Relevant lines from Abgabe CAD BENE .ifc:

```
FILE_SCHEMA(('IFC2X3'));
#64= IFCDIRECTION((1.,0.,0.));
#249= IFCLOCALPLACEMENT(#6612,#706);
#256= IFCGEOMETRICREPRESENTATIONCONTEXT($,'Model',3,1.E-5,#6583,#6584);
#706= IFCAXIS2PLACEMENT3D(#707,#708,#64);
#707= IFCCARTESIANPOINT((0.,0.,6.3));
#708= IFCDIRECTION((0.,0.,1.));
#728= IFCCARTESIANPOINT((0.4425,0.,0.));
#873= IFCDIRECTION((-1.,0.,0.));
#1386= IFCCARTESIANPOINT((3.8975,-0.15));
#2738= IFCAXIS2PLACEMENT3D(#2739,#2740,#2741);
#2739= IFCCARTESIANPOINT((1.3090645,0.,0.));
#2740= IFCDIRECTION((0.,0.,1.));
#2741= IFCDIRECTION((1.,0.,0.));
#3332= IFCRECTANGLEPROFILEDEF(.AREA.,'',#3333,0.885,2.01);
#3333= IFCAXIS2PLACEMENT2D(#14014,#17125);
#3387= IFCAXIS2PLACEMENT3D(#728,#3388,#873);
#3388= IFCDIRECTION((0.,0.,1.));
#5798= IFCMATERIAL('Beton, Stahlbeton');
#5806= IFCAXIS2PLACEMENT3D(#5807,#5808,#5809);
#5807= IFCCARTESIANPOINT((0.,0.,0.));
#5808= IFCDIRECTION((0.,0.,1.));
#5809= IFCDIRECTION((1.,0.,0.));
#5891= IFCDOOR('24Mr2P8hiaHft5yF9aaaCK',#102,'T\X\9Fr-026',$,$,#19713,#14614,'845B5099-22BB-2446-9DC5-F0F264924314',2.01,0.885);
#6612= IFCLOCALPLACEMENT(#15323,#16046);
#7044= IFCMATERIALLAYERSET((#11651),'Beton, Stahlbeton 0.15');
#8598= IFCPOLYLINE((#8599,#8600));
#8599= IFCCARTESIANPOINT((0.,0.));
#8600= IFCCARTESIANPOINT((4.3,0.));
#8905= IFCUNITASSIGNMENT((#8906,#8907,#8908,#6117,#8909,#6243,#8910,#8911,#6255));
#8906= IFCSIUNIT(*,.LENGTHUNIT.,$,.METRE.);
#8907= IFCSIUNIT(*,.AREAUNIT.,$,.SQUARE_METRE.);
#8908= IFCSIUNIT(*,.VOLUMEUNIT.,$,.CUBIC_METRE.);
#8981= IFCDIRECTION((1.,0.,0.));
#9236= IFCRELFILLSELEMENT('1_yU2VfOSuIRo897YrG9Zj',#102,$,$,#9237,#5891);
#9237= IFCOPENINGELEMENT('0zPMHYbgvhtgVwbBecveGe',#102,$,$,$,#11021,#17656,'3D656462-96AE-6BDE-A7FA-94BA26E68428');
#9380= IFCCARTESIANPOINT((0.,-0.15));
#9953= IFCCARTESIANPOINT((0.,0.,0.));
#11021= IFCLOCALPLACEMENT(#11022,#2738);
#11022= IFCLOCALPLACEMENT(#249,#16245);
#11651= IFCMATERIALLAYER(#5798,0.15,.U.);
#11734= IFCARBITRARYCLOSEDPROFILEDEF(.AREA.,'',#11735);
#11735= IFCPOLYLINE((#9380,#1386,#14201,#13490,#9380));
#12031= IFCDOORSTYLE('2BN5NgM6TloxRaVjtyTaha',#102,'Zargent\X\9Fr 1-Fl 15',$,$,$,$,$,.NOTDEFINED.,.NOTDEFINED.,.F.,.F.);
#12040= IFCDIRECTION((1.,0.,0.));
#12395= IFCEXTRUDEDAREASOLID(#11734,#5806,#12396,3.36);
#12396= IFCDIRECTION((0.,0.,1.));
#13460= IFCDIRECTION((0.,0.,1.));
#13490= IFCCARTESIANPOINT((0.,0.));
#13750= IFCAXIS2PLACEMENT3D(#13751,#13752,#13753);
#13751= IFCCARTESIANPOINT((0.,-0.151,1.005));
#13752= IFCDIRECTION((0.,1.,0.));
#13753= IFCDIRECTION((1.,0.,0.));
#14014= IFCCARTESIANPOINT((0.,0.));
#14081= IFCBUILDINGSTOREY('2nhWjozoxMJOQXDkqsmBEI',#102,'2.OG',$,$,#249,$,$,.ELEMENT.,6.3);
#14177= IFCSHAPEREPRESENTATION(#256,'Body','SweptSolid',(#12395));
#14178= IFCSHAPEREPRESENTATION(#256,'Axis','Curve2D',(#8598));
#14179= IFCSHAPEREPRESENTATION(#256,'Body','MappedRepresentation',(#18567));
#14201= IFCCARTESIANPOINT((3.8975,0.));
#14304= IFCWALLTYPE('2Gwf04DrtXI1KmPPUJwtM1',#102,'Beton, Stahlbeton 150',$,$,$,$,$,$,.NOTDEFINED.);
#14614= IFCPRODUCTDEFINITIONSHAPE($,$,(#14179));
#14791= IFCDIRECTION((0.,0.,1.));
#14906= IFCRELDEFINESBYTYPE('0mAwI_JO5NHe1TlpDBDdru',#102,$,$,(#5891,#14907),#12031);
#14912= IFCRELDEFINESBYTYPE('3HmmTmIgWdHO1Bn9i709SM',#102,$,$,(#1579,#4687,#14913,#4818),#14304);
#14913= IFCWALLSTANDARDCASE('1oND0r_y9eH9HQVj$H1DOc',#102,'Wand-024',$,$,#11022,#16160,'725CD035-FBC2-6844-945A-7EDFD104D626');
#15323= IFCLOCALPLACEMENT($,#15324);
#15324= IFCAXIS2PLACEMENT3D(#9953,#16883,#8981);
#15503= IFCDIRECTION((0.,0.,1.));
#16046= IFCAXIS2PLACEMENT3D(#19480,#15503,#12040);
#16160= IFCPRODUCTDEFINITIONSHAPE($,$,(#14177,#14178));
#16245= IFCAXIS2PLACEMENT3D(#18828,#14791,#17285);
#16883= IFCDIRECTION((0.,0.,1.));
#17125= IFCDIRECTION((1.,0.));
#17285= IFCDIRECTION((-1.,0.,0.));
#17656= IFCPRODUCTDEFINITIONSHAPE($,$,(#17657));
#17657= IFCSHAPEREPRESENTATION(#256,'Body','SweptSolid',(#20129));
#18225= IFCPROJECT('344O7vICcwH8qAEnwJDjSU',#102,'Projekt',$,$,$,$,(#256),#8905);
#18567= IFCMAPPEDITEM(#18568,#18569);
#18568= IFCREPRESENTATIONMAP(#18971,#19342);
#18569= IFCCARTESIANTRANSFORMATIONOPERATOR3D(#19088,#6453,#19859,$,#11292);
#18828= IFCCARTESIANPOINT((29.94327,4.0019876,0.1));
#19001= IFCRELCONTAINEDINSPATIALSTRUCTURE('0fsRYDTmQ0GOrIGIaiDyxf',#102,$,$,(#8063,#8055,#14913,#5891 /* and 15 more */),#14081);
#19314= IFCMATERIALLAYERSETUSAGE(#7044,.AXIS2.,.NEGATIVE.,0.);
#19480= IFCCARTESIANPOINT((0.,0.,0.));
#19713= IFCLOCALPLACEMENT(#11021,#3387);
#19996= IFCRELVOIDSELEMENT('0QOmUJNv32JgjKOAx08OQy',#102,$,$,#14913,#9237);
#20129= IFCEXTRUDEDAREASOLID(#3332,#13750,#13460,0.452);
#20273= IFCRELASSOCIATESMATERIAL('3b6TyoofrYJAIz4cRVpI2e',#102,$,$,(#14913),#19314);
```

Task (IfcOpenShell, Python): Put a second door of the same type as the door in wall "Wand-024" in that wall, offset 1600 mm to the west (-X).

```python
import ifcopenshell
import ifcopenshell.api.feature
import ifcopenshell.api.geometry
import ifcopenshell.api.root
import ifcopenshell.geom
import ifcopenshell.util.element
import ifcopenshell.util.placement
import ifcopenshell.util.shape

model = ifcopenshell.open("Abgabe CAD BENE .ifc")
settings = ifcopenshell.geom.settings()


def volume(element):
    """Net volume in cubic metres, openings subtracted."""
    shape = ifcopenshell.geom.create_shape(settings, element)
    return ifcopenshell.util.shape.get_volume(shape.geometry)


def reuse_history(source, copy):
    """copy_class also copies each property set's owner history, people and application; keep the originals."""
    for rel in copy.IsDefinedBy:
        if rel.is_a("IfcRelDefinesByProperties") and (history := rel.RelatingPropertyDefinition.OwnerHistory):
            rel.RelatingPropertyDefinition.OwnerHistory = source.OwnerHistory
            ifcopenshell.util.element.remove_deep2(model, history)


door = model.by_guid("24Mr2P8hiaHft5yF9aaaCK")
opening = door.FillsVoids[0].RelatingOpeningElement
wall = opening.VoidsElements[0].RelatingBuildingElement
before = volume(wall)
shift = ifcopenshell.util.placement.get_local_placement(wall.ObjectPlacement)[:3, 0] * 1.6

# copy_class copies the void relationship, type, container and properties, but no geometry.
new_opening = ifcopenshell.api.root.copy_class(model, product=opening)
new_opening.Representation = ifcopenshell.util.element.copy_deep(
    model, opening.Representation, exclude=["IfcGeometricRepresentationContext", "IfcRepresentationMap"]
)
new_opening.Tag = None
new_door = ifcopenshell.api.root.copy_class(model, product=door)
new_door.Representation = ifcopenshell.util.element.copy_deep(
    model, door.Representation, exclude=["IfcGeometricRepresentationContext", "IfcRepresentationMap"]
)
new_door.Tag = None
reuse_history(door, new_door)
fills = ifcopenshell.api.feature.add_filling(model, opening=new_opening, element=new_door)
fills.OwnerHistory = new_door.OwnerHistory  # required in IFC2X3

for old, new in ((opening, new_opening), (door, new_door)):
    matrix = ifcopenshell.util.placement.get_local_placement(old.ObjectPlacement)
    matrix[:3, 3] += shift
    ifcopenshell.api.geometry.edit_object_placement(model, product=new, matrix=matrix, is_si=False)

after = volume(wall)

print(f"wall volume {before:.3f} -> {after:.3f} m3")

model.write("Abgabe CAD BENE _edited.ifc")
```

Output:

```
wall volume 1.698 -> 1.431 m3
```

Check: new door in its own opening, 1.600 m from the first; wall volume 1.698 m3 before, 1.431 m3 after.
